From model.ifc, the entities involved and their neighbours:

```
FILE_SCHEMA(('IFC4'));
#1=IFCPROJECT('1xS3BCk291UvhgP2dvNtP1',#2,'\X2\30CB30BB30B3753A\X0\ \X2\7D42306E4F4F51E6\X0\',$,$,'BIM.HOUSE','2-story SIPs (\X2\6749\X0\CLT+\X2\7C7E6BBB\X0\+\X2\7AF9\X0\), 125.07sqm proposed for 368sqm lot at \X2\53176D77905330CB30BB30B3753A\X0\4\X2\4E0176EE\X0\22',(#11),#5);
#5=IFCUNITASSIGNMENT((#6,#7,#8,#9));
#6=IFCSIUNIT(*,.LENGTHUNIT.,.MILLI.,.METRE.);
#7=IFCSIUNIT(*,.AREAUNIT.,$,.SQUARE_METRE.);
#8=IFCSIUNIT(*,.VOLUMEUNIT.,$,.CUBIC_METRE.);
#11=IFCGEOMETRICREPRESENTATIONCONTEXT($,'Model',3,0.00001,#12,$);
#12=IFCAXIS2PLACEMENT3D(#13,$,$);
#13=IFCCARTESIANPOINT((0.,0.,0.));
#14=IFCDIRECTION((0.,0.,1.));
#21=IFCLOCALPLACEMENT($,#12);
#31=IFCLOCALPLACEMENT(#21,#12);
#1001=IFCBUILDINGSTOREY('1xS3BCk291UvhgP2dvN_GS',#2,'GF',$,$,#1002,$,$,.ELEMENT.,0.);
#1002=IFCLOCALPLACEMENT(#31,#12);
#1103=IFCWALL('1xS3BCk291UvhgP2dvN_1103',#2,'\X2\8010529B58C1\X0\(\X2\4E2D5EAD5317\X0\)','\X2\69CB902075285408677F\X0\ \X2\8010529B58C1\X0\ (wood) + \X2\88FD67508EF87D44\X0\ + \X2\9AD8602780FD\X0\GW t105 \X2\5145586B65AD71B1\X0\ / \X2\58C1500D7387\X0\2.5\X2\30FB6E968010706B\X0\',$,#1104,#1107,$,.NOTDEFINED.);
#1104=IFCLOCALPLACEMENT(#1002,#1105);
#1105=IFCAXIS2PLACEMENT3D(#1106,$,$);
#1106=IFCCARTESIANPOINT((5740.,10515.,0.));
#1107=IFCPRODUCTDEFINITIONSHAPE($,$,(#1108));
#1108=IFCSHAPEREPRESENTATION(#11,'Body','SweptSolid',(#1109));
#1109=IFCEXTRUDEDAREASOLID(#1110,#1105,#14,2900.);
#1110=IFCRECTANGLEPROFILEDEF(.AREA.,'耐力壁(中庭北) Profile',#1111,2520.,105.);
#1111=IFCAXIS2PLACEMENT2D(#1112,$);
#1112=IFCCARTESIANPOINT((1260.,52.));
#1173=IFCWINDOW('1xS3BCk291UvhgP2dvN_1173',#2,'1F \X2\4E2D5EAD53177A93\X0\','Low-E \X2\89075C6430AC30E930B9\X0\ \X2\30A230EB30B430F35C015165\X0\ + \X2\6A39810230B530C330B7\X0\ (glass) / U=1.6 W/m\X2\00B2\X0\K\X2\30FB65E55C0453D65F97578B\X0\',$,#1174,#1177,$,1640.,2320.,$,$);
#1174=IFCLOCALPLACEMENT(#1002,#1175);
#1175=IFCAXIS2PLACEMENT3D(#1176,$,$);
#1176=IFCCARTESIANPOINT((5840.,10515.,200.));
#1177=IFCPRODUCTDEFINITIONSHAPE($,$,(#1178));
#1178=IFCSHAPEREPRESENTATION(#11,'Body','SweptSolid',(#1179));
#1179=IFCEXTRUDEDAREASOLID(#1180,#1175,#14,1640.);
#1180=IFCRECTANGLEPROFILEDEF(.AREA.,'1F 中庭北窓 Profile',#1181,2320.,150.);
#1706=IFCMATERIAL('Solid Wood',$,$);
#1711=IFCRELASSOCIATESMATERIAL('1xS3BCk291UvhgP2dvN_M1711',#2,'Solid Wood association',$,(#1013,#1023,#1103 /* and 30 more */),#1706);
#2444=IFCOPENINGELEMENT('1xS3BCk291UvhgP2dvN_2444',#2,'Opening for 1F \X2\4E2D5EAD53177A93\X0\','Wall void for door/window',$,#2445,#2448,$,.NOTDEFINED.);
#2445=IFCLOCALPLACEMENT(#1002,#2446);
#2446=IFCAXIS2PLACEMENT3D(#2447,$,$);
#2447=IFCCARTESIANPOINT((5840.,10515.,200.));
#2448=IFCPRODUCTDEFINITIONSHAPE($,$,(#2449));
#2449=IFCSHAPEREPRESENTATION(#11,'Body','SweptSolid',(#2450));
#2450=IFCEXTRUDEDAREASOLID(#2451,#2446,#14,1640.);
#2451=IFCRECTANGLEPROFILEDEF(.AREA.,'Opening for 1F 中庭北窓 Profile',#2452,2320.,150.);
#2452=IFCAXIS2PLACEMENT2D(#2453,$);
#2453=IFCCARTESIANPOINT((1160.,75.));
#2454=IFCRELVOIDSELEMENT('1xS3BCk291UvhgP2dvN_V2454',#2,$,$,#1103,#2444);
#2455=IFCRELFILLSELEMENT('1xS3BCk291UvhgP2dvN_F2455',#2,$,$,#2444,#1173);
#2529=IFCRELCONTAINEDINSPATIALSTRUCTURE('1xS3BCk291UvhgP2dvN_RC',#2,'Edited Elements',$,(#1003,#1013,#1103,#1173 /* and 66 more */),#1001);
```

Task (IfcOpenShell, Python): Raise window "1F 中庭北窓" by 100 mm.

```python
import numpy as np
import ifcopenshell
import ifcopenshell.api.geometry
import ifcopenshell.util.placement
import ifcopenshell.util.unit

model = ifcopenshell.open("model.ifc")
unit_scale = ifcopenshell.util.unit.calculate_unit_scale(model)

window = model.by_guid("1xS3BCk291UvhgP2dvN_1173")
opening = window.FillsVoids[0].RelatingOpeningElement
dz = 100.0

shift = np.array([0.0, 0.0, dz])
# The window is not placed relative to its opening, so move both.
for product in (opening, window):
    matrix = ifcopenshell.util.placement.get_local_placement(product.ObjectPlacement)
    matrix[:3, 3] += shift
    ifcopenshell.api.geometry.edit_object_placement(model, product=product, matrix=matrix, is_si=False)

print(f"moved by {dz * unit_scale:+.3f} m")

model.write("model_rev.ifc")
```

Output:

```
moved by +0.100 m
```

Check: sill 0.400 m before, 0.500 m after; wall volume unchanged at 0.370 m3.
